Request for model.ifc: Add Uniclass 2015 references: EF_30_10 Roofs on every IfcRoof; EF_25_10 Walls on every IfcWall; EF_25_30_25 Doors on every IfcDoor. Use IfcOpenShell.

First a look at what the model holds.

```python
import ifcopenshell

model = ifcopenshell.open("model.ifc")
print(model.schema)
print("classifications:", [c.Name for c in model.by_type("IfcClassification")])
for ifc_class in ("IfcDoor", "IfcRoof", "IfcStair", "IfcWall", "IfcWindow"):
    print(ifc_class, len(model.by_type(ifc_class)))
```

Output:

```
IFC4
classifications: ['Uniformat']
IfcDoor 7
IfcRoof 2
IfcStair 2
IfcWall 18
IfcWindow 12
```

```python
import ifcopenshell
import ifcopenshell.api.classification

model = ifcopenshell.open("model.ifc")

system = ifcopenshell.api.classification.add_classification(model, classification="Uniclass 2015")

codes = {
    "IfcRoof": ("EF_30_10", "Roofs"),
    "IfcWall": ("EF_25_10", "Walls"),
    "IfcDoor": ("EF_25_30_25", "Doors"),
}
for ifc_class, (code, name) in codes.items():
    products = model.by_type(ifc_class)
    ifcopenshell.api.classification.add_reference(
        model, products=products, classification=system, identification=code, name=name
    )
    print(code, len(products))

model.write("model_updated.ifc")
```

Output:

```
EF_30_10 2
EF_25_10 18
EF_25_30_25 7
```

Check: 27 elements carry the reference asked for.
